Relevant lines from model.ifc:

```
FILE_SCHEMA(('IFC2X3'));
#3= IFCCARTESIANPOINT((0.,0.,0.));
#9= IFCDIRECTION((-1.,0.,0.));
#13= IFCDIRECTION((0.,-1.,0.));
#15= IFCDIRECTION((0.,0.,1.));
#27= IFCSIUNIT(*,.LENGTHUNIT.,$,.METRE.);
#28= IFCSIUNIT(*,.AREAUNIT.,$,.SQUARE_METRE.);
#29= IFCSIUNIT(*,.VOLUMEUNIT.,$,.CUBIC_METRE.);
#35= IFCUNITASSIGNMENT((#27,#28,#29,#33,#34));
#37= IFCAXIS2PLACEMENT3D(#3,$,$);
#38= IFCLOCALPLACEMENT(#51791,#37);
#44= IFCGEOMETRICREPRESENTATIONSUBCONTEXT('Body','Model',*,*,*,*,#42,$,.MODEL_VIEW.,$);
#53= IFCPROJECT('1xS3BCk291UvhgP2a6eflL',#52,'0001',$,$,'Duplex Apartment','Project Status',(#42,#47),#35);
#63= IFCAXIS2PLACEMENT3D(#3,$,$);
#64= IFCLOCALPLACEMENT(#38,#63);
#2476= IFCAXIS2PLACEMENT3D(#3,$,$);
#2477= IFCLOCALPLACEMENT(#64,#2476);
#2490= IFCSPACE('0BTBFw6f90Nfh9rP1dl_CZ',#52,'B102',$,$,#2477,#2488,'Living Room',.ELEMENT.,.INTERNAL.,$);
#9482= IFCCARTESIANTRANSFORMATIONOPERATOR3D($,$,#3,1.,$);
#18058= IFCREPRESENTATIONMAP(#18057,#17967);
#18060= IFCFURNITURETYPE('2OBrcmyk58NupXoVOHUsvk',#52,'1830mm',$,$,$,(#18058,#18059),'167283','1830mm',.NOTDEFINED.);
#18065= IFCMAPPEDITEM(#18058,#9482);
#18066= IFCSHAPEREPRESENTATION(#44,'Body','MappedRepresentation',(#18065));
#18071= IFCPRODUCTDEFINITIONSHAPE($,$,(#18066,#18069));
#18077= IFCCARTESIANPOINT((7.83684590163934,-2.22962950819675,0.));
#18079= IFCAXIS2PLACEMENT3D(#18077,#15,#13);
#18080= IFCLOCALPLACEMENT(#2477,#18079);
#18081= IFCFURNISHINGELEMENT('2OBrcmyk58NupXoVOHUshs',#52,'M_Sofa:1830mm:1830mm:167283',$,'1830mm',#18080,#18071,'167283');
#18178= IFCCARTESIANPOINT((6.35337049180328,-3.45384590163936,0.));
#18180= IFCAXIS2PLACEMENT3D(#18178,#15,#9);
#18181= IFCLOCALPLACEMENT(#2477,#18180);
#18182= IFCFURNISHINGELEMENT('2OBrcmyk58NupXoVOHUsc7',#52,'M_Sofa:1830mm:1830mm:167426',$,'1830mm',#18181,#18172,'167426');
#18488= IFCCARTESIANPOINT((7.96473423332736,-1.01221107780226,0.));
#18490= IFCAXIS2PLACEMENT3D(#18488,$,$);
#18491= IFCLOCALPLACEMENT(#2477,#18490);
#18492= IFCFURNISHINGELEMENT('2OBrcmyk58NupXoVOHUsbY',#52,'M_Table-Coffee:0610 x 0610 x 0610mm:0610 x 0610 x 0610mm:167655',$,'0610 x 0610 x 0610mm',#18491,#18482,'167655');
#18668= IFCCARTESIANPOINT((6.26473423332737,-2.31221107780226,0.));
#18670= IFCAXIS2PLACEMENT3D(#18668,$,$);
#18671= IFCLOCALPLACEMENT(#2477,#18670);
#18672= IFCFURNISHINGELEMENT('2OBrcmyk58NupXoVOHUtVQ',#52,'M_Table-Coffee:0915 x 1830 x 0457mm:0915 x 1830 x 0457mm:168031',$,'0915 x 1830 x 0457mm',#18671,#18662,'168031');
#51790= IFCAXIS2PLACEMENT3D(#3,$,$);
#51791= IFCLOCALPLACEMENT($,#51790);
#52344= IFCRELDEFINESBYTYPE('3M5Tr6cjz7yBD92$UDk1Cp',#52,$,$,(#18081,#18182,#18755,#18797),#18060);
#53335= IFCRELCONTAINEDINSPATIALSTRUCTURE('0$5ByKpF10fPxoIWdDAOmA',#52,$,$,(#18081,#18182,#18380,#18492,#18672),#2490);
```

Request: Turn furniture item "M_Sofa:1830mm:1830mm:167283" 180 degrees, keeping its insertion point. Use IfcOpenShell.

```python
import ifcopenshell
import ifcopenshell.api.geometry
import ifcopenshell.util.placement

model = ifcopenshell.open("model.ifc")

item = model.by_id(18081)
matrix = ifcopenshell.util.placement.get_local_placement(item.ObjectPlacement)
matrix = matrix @ ifcopenshell.util.placement.rotation(180, "Z")
ifcopenshell.api.geometry.edit_object_placement(model, product=item, matrix=matrix, is_si=False)

print(ifcopenshell.util.placement.get_local_placement(item.ObjectPlacement).round(3) + 0.0)

model.write("model_updated.ifc")
```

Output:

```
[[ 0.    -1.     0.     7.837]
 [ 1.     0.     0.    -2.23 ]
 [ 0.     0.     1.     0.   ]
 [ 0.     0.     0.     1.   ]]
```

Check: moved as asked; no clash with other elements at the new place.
